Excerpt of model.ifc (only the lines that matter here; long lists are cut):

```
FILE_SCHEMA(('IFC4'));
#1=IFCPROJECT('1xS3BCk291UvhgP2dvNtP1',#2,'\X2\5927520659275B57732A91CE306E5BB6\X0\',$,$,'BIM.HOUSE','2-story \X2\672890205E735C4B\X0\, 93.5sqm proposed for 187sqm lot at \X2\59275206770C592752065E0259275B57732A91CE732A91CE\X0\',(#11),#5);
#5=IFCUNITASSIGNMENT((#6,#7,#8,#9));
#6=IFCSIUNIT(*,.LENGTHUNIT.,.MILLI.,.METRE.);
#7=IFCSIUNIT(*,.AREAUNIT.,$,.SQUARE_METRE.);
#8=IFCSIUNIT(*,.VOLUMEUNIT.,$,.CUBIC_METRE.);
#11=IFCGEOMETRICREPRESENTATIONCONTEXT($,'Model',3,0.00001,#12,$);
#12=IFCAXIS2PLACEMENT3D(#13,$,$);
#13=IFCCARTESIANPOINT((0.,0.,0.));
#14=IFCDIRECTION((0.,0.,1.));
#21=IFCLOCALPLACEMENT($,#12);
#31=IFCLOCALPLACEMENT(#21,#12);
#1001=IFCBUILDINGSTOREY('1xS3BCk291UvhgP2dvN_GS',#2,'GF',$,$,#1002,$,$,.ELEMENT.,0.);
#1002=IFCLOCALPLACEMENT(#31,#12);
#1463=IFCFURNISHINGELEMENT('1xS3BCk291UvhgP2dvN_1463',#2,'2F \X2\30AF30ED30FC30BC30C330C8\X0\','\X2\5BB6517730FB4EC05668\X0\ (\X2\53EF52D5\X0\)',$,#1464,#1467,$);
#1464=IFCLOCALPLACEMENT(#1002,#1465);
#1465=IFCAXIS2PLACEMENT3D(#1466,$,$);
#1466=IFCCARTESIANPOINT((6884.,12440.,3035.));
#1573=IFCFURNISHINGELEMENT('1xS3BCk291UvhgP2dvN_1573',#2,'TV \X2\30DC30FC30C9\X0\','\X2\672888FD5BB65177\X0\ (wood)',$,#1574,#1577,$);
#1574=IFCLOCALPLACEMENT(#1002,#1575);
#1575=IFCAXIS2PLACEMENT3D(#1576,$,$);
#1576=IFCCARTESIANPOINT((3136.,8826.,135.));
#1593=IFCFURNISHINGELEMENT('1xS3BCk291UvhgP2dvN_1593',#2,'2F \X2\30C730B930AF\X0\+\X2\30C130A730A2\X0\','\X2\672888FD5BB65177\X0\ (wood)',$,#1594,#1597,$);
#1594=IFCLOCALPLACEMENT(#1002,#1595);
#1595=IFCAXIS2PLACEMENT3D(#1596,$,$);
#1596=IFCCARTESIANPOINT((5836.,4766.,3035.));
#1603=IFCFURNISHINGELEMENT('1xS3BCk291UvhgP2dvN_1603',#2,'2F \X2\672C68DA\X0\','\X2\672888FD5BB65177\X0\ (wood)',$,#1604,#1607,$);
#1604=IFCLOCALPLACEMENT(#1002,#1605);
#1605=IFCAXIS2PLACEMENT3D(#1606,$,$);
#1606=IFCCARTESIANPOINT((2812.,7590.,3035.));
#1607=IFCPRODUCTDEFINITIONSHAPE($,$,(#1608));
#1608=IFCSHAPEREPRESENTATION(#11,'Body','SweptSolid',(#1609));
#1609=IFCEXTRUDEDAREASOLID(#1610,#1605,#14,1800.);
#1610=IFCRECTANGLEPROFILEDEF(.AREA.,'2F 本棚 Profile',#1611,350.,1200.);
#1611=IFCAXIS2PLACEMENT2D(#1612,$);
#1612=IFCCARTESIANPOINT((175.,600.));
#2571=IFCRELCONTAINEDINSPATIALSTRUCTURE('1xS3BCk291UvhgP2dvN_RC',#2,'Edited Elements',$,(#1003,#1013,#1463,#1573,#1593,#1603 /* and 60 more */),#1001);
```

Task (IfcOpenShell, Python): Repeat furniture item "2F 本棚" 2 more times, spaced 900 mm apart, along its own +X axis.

```python
import ifcopenshell
import ifcopenshell.api.geometry
import ifcopenshell.api.root
import ifcopenshell.util.element
import ifcopenshell.util.placement
import ifcopenshell.util.unit

model = ifcopenshell.open("model.ifc")
unit_scale = ifcopenshell.util.unit.calculate_unit_scale(model)


def reuse_history(source, copy):
    """copy_class also copies each property set's owner history, people and application; keep the originals."""
    for rel in copy.IsDefinedBy:
        if rel.is_a("IfcRelDefinesByProperties") and (history := rel.RelatingPropertyDefinition.OwnerHistory):
            rel.RelatingPropertyDefinition.OwnerHistory = source.OwnerHistory
            ifcopenshell.util.element.remove_deep2(model, history)


source = model.by_guid("1xS3BCk291UvhgP2dvN_1603")
base = ifcopenshell.util.placement.get_local_placement(source.ObjectPlacement)
step = base[:3, 0] * 0.9 / unit_scale

for i in range(1, 3):
    copy = ifcopenshell.api.root.copy_class(model, product=source)
    copy.Representation = ifcopenshell.util.element.copy_deep(
        model, source.Representation, exclude=["IfcGeometricRepresentationContext", "IfcRepresentationMap"]
    )
    reuse_history(source, copy)
    matrix = base.copy()
    matrix[:3, 3] += i * step
    print("added at", matrix[:3, 3].round(3) + 0.0)
    ifcopenshell.api.geometry.edit_object_placement(model, product=copy, matrix=matrix, is_si=False)

model.write("model_edited.ifc")
```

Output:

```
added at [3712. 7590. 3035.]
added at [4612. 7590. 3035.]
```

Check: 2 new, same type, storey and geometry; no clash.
